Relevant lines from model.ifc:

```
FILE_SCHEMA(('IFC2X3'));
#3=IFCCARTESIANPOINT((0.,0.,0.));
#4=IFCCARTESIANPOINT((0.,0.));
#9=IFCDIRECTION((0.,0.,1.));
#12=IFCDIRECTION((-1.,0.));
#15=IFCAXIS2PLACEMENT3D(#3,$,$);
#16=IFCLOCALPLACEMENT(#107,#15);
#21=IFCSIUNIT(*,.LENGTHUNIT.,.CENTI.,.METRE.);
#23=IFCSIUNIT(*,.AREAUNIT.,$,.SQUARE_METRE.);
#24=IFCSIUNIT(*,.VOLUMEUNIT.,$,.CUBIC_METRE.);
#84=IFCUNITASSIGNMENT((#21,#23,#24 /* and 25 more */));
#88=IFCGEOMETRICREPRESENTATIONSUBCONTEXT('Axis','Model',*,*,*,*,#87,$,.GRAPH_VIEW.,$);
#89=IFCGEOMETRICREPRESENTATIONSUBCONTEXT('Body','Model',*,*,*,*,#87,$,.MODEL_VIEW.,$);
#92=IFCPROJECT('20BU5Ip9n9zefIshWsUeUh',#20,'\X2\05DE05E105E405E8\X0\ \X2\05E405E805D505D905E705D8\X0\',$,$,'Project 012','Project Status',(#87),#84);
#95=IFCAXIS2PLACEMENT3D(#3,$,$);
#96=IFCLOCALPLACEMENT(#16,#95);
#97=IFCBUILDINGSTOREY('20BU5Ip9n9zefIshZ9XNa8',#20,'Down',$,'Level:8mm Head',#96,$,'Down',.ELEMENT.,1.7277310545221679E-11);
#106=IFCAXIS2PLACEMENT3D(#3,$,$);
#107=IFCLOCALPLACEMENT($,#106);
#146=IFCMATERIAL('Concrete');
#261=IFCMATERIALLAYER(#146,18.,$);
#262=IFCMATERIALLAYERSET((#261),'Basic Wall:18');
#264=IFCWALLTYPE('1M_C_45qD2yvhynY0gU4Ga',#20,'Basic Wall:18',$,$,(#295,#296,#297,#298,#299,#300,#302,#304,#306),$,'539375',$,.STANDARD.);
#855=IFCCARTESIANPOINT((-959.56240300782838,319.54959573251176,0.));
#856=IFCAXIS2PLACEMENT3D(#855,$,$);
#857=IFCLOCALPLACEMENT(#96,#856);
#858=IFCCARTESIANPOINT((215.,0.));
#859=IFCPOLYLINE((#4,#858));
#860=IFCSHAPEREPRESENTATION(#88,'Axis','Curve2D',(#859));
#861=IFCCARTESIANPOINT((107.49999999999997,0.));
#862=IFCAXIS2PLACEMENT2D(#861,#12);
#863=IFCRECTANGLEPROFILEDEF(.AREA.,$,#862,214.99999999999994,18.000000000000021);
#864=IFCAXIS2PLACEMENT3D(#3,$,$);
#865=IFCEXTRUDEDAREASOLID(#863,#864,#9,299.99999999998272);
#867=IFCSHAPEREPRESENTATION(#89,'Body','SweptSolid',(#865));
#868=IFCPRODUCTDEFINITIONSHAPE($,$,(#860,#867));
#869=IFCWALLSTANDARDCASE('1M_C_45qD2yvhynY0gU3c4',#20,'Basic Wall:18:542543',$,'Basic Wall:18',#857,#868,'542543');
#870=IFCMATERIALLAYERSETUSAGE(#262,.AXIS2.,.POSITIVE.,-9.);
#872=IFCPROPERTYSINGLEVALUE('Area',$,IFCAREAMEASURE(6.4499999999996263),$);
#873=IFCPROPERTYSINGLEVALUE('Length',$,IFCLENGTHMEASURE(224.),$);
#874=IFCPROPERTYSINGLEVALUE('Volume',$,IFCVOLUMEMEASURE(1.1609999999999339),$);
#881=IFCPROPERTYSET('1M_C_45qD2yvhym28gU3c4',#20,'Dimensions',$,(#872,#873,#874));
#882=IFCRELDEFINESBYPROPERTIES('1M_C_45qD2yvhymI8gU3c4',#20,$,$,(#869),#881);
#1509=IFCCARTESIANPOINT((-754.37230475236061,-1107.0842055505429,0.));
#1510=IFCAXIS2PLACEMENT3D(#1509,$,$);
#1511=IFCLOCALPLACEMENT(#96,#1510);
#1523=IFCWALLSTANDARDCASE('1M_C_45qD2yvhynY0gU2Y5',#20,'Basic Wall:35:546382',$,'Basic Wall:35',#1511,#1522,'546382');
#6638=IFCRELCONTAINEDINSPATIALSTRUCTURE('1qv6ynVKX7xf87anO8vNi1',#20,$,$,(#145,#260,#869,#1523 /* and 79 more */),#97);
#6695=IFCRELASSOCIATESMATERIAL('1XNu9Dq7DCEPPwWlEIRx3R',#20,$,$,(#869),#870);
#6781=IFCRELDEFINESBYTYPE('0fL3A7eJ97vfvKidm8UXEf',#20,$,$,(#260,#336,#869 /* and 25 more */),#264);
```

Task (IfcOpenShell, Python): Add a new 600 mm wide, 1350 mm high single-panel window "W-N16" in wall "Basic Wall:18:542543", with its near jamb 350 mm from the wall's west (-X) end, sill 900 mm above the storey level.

```python
import numpy as np
import ifcopenshell
import ifcopenshell.api.feature
import ifcopenshell.api.geometry
import ifcopenshell.api.pset
import ifcopenshell.api.root
import ifcopenshell.api.spatial
import ifcopenshell.api.type
import ifcopenshell.geom
import ifcopenshell.util.element
import ifcopenshell.util.placement
import ifcopenshell.util.representation
import ifcopenshell.util.shape
import ifcopenshell.util.unit

model = ifcopenshell.open("model.ifc")
unit_scale = ifcopenshell.util.unit.calculate_unit_scale(model)
area_scale = ifcopenshell.util.unit.calculate_unit_scale(model, "AREAUNIT")
volume_scale = ifcopenshell.util.unit.calculate_unit_scale(model, "VOLUMEUNIT")
settings = ifcopenshell.geom.settings()


def volume(element):
    """Net volume in cubic metres, openings subtracted."""
    shape = ifcopenshell.geom.create_shape(settings, element)
    return ifcopenshell.util.shape.get_volume(shape.geometry)


wall = model.by_id(869)
storey = ifcopenshell.util.element.get_container(wall, ifc_class="IfcBuildingStorey")
context = ifcopenshell.util.representation.get_context(model, "Model", "Body", "MODEL_VIEW")
before = volume(wall)

width, height, from_end, sill = 0.6, 1.35, 0.35, 0.9  # metres

# The wall runs along its own X axis, and the end named is its -X end.
wall_shape = ifcopenshell.geom.create_shape(settings, wall)
x, y, z = ifcopenshell.util.shape.get_vertices(wall_shape.geometry).T
start = x.min() + from_end
face, thickness = float(y.min()), float(y.max() - y.min())
wall_matrix = ifcopenshell.util.placement.get_local_placement(wall.ObjectPlacement)
level = ifcopenshell.util.placement.get_local_placement(storey.ObjectPlacement)[2, 3]


def in_wall(x, y):
    """Placement at x, y metres in the wall's axes, at sill height."""
    matrix = wall_matrix.copy()
    matrix[:, 3] = wall_matrix @ np.array([x / unit_scale, y / unit_scale, 0.0, 1.0])
    matrix[2, 3] = level + sill / unit_scale
    return matrix


# Opening: a box that overshoots both wall faces by 50 mm.
opening = ifcopenshell.api.root.create_entity(model, ifc_class="IfcOpeningElement")
box = ifcopenshell.api.geometry.add_wall_representation(
    model, context=context, length=width, height=height, thickness=thickness + 0.1
)
ifcopenshell.api.geometry.assign_representation(model, product=opening, representation=box)
ifcopenshell.api.geometry.edit_object_placement(model, product=opening, matrix=in_wall(start, face - 0.05), is_si=False)
ifcopenshell.api.feature.add_feature(model, feature=opening, element=wall)

window = ifcopenshell.api.root.create_entity(model, ifc_class="IfcWindow", name="W-N16")
window.OverallWidth, window.OverallHeight = width / unit_scale, height / unit_scale
body = ifcopenshell.api.geometry.add_window_representation(
    model,
    context=context,
    overall_width=window.OverallWidth,
    overall_height=window.OverallHeight,
    partition_type="SINGLE_PANEL",
)
ifcopenshell.api.geometry.assign_representation(model, product=window, representation=body)
ifcopenshell.api.spatial.assign_container(model, products=[window], relating_structure=storey)
fills = ifcopenshell.api.feature.add_filling(model, opening=opening, element=window)
fills.OwnerHistory = window.OwnerHistory  # required in IFC2X3

# IFC2X3 keeps the operation on the window style.
style = ifcopenshell.api.root.create_entity(model, ifc_class="IfcWindowStyle", name="W-N16")
style.OperationType, style.ConstructionType = "SINGLE_PANEL", "NOTDEFINED"
style.ParameterTakesPrecedence = style.Sizeable = False
ifcopenshell.api.type.assign_type(model, related_objects=[window], relating_type=style)

# Centre the window in the wall's thickness.
ifcopenshell.api.geometry.edit_object_placement(model, product=window, matrix=in_wall(start, face), is_si=False)
window_shape = ifcopenshell.geom.create_shape(settings, window)
depth = ifcopenshell.util.shape.get_vertices(window_shape.geometry)[:, 1]
offset = face + thickness / 2 - (depth.min() + depth.max()) / 2
ifcopenshell.api.geometry.edit_object_placement(model, product=window, matrix=in_wall(start, offset), is_si=False)

after = volume(wall)

# Update the wall's stored quantities.
pset = model.by_id(ifcopenshell.util.element.get_pset(wall, "Dimensions", should_inherit=False)["id"])
ifcopenshell.api.pset.edit_pset(model, pset=pset, properties={
    "Area": model.create_entity("IfcAreaMeasure", after / thickness / area_scale),
    "Volume": model.create_entity("IfcVolumeMeasure", after / volume_scale),
})

print(f"wall volume {before:.3f} -> {after:.3f} m3")

model.write("model_v2.ifc")
```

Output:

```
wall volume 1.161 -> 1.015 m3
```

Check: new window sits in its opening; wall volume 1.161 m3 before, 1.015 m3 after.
